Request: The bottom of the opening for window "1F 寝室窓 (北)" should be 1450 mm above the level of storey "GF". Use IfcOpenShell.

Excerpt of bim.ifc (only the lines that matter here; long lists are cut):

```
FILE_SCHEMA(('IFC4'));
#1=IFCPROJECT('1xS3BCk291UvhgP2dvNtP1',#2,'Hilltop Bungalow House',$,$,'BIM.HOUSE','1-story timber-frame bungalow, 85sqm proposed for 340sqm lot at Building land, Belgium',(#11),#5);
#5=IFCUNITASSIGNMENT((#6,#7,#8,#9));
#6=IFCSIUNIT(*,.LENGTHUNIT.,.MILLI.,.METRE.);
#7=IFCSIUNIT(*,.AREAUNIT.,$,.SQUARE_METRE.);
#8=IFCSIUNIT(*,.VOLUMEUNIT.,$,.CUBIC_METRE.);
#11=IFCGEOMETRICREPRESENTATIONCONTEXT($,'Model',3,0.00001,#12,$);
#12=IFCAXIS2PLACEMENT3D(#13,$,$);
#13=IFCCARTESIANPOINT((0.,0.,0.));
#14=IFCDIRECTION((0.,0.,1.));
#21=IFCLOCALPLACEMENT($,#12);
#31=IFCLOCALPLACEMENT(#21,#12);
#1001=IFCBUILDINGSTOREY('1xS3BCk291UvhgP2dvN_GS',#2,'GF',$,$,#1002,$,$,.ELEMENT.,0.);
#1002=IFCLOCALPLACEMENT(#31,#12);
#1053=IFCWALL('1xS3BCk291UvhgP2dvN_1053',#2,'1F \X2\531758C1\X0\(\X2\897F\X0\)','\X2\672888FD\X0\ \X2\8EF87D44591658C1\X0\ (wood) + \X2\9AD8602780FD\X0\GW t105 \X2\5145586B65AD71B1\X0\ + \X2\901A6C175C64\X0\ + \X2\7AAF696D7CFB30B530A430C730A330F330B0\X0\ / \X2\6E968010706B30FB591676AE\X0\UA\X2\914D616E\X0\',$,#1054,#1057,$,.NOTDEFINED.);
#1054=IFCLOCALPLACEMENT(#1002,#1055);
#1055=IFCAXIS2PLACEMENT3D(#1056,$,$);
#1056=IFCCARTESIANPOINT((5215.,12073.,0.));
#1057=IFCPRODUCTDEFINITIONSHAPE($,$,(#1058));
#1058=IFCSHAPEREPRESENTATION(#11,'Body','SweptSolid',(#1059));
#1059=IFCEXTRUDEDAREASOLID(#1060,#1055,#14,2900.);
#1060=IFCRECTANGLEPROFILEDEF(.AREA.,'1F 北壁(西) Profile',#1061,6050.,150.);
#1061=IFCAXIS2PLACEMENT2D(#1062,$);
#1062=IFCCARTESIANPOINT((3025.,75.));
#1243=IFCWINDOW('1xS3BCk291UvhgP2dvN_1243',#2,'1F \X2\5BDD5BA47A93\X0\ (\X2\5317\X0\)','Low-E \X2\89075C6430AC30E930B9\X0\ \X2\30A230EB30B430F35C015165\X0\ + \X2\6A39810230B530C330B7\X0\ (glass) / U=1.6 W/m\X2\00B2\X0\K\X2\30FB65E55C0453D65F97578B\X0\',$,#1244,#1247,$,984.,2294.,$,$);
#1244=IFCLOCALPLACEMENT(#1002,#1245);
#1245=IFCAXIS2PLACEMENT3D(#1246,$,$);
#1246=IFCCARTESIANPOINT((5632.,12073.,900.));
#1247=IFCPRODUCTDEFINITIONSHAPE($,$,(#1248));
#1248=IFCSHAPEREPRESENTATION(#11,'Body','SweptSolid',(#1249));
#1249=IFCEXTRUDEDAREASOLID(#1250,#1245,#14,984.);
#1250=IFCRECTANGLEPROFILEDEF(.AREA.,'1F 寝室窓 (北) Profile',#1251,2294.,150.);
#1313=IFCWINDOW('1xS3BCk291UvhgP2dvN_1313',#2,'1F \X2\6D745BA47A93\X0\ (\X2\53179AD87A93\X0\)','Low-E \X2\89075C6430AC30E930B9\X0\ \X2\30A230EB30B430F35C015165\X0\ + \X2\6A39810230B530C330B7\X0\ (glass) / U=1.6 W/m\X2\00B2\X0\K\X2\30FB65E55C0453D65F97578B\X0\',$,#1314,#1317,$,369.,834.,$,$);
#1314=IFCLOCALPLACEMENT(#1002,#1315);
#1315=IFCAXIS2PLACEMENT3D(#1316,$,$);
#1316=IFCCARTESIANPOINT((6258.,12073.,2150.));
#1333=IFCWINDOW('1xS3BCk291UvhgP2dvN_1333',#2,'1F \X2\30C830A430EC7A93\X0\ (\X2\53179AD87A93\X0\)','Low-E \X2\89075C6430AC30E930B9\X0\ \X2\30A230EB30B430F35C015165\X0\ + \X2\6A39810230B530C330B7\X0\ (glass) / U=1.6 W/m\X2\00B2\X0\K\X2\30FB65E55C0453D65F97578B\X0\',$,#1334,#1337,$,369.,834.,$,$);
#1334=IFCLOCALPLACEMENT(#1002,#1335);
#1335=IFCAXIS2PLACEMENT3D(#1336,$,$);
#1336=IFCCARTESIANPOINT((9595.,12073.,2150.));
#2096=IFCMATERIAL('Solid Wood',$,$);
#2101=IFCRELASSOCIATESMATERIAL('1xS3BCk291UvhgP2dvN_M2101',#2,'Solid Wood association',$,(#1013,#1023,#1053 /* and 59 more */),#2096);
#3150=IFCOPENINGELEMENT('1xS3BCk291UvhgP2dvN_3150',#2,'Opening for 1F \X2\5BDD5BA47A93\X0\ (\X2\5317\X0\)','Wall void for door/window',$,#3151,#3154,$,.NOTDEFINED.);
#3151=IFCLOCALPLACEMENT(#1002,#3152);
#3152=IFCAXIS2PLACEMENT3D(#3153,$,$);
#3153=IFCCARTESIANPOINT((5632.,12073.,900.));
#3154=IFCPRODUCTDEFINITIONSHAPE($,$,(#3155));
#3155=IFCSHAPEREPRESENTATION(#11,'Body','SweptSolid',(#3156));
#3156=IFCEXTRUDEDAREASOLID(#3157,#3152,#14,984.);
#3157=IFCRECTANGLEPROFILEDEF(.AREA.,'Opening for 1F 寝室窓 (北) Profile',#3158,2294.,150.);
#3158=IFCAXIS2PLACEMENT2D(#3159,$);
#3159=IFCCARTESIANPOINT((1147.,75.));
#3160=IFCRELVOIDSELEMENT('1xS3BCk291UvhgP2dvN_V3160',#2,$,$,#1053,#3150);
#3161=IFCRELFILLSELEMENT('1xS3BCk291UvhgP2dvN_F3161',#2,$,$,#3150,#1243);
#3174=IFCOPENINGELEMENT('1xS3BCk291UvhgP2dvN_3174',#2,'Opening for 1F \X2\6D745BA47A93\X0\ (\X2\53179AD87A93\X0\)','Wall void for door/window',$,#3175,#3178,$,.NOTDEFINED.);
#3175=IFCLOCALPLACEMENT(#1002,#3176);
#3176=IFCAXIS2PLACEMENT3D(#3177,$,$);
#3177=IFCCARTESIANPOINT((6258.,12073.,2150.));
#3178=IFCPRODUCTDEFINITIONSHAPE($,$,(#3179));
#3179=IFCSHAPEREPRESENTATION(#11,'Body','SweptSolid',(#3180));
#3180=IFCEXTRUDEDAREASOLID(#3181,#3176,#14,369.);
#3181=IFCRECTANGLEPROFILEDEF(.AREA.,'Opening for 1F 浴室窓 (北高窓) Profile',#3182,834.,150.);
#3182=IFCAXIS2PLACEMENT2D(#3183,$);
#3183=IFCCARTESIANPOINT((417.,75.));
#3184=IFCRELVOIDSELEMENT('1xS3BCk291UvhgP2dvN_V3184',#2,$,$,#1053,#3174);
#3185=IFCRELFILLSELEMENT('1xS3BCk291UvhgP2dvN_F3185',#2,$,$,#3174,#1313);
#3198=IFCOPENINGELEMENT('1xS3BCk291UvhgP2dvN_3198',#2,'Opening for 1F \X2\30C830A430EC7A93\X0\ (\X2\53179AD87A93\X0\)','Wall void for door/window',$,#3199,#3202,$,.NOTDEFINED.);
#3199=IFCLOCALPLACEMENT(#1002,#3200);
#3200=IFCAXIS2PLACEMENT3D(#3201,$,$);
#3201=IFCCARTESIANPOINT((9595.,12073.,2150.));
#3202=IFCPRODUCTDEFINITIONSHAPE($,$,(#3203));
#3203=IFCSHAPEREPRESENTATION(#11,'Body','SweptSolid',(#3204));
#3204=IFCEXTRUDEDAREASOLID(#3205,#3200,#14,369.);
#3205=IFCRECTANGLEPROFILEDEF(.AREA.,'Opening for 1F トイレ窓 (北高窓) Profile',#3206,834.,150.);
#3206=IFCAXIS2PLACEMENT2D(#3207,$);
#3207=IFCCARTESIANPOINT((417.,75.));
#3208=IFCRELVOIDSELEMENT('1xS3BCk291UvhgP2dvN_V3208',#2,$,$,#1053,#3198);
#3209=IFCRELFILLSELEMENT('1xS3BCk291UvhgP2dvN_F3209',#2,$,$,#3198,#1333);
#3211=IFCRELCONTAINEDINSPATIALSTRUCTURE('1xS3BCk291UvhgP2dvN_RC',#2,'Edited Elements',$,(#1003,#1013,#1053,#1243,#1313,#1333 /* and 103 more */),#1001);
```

```python
import numpy as np
import ifcopenshell
import ifcopenshell.api.geometry
import ifcopenshell.geom
import ifcopenshell.util.element
import ifcopenshell.util.placement
import ifcopenshell.util.shape
import ifcopenshell.util.unit

model = ifcopenshell.open("bim.ifc")
unit_scale = ifcopenshell.util.unit.calculate_unit_scale(model)

window = model.by_guid("1xS3BCk291UvhgP2dvN_1243")
opening = window.FillsVoids[0].RelatingOpeningElement
storey = ifcopenshell.util.element.get_container(window, ifc_class="IfcBuildingStorey")
level = ifcopenshell.util.placement.get_local_placement(storey.ObjectPlacement)[2, 3]

# The opening's origin need not be at the sill, so measure its lowest point.
shape = ifcopenshell.geom.create_shape(ifcopenshell.geom.settings(), opening)
bottom = ifcopenshell.util.shape.get_shape_bottom_elevation(shape, shape.geometry) / unit_scale
dz = level + 1.45 / unit_scale - bottom

shift = np.array([0.0, 0.0, dz])
# The window is not placed relative to its opening, so move both.
for product in (opening, window):
    matrix = ifcopenshell.util.placement.get_local_placement(product.ObjectPlacement)
    matrix[:3, 3] += shift
    ifcopenshell.api.geometry.edit_object_placement(model, product=product, matrix=matrix, is_si=False)

print(f"moved by {dz * unit_scale:+.3f} m")

model.write("bim_v2.ifc")
```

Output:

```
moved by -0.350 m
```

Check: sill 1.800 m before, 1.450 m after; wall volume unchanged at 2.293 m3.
